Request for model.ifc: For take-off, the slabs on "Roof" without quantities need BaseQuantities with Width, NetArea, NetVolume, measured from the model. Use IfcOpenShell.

First a look at what the model holds.

```python
import ifcopenshell
import ifcopenshell.util.element
import ifcopenshell.util.unit

model = ifcopenshell.open("model.ifc")
print(model.schema)
for unit_type in ("LENGTHUNIT", "AREAUNIT", "VOLUMEUNIT"):
    print(unit_type, ifcopenshell.util.unit.calculate_unit_scale(model, unit_type))
storey = next(s for s in model.by_type("IfcBuildingStorey") if s.Name == "Roof")
slabs = [e for e in ifcopenshell.util.element.get_decomposition(storey) if e.is_a("IfcSlab")]
for e in sorted(slabs, key=lambda e: e.id()):
    print(e.id(), e.is_a(), e.Name, list(ifcopenshell.util.element.get_psets(e, qtos_only=True)), sep=" | ")
```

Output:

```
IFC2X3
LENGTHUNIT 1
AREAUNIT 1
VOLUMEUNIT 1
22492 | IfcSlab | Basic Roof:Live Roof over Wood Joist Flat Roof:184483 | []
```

```python
import ifcopenshell
import ifcopenshell.api.pset
import ifcopenshell.geom
import ifcopenshell.util.element
import ifcopenshell.util.shape
import ifcopenshell.util.unit

model = ifcopenshell.open("model.ifc")
unit_scale = ifcopenshell.util.unit.calculate_unit_scale(model)
area_scale = ifcopenshell.util.unit.calculate_unit_scale(model, "AREAUNIT")
volume_scale = ifcopenshell.util.unit.calculate_unit_scale(model, "VOLUMEUNIT")
settings = ifcopenshell.geom.settings()

storey = next(s for s in model.by_type("IfcBuildingStorey") if s.Name == "Roof")
slabs = [e for e in ifcopenshell.util.element.get_decomposition(storey) if e.is_a("IfcSlab")]

for e in sorted(slabs, key=lambda e: e.id()):
    if ifcopenshell.util.element.get_psets(e, qtos_only=True, should_inherit=False):
        continue
    # Geometry comes back in metres, in the element's own axes.
    shape = ifcopenshell.geom.create_shape(settings, e)
    values = {
        "Width": ifcopenshell.util.shape.get_z(shape.geometry) / unit_scale,
        "NetArea": ifcopenshell.util.shape.get_footprint_area(shape.geometry) / area_scale,
        "NetVolume": ifcopenshell.util.shape.get_volume(shape.geometry) / volume_scale,
    }
    qto = ifcopenshell.api.pset.add_qto(model, product=e, name="BaseQuantities")
    ifcopenshell.api.pset.edit_qto(model, qto=qto, properties=values)
    print(e.id(), {k: round(v, 3) for k, v in values.items()})

model.write("model-out.ifc")
```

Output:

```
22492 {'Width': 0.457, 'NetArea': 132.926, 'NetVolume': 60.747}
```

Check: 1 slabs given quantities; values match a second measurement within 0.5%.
